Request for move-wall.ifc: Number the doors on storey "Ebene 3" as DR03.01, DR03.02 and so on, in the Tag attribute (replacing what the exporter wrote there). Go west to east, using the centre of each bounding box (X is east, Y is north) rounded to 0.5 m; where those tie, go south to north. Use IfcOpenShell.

First a look at what the model holds.

```python
import ifcopenshell
import ifcopenshell.util.element
import ifcopenshell.util.placement

model = ifcopenshell.open("move-wall.ifc")
print(model.schema)
storey = next(s for s in model.by_type("IfcBuildingStorey") if s.Name == "Ebene 3")
doors = [e for e in ifcopenshell.util.element.get_decomposition(storey) if e.is_a("IfcDoor")]
for e in sorted(doors, key=lambda e: e.id()):
    origin = ifcopenshell.util.placement.get_local_placement(e.ObjectPlacement)[:3, 3]
    print(e.id(), e.Tag, e.Name, origin.round(2) + 0.0, sep=" | ")
```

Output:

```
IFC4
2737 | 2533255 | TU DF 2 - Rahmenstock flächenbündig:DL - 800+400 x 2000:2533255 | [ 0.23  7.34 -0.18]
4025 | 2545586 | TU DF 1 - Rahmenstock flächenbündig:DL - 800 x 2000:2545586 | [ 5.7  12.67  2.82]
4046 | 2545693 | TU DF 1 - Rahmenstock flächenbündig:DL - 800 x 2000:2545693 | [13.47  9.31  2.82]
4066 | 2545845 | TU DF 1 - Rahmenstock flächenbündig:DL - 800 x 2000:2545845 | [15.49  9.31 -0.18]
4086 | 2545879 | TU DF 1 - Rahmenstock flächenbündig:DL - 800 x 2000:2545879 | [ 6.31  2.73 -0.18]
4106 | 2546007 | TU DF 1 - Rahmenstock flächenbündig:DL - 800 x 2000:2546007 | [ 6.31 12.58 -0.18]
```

```python
import ifcopenshell
import ifcopenshell.geom
import ifcopenshell.util.element
import ifcopenshell.util.shape

model = ifcopenshell.open("move-wall.ifc")
settings = ifcopenshell.geom.settings()
settings.set("use-world-coords", True)


def centre(element):
    shape = ifcopenshell.geom.create_shape(settings, element)
    return ifcopenshell.util.shape.get_bbox_centroid(shape.geometry)


storey = next(s for s in model.by_type("IfcBuildingStorey") if s.Name == "Ebene 3")
doors = [e for e in ifcopenshell.util.element.get_decomposition(storey) if e.is_a("IfcDoor")]

# Insertion points can sit at a corner or the storey origin, so sort by the geometry (in metres).
centres = {e: centre(e) for e in doors}
doors.sort(key=lambda e: (round(centres[e][0] / 0.5), centres[e][1]))

for i, e in enumerate(doors, start=1):
    number = f"DR03.{i:02d}"
    e.Tag = number
    print(e.id(), number)

model.write("move-wall-out.ifc")
```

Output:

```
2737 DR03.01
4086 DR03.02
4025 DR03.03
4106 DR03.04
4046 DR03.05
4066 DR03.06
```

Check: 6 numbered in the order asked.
